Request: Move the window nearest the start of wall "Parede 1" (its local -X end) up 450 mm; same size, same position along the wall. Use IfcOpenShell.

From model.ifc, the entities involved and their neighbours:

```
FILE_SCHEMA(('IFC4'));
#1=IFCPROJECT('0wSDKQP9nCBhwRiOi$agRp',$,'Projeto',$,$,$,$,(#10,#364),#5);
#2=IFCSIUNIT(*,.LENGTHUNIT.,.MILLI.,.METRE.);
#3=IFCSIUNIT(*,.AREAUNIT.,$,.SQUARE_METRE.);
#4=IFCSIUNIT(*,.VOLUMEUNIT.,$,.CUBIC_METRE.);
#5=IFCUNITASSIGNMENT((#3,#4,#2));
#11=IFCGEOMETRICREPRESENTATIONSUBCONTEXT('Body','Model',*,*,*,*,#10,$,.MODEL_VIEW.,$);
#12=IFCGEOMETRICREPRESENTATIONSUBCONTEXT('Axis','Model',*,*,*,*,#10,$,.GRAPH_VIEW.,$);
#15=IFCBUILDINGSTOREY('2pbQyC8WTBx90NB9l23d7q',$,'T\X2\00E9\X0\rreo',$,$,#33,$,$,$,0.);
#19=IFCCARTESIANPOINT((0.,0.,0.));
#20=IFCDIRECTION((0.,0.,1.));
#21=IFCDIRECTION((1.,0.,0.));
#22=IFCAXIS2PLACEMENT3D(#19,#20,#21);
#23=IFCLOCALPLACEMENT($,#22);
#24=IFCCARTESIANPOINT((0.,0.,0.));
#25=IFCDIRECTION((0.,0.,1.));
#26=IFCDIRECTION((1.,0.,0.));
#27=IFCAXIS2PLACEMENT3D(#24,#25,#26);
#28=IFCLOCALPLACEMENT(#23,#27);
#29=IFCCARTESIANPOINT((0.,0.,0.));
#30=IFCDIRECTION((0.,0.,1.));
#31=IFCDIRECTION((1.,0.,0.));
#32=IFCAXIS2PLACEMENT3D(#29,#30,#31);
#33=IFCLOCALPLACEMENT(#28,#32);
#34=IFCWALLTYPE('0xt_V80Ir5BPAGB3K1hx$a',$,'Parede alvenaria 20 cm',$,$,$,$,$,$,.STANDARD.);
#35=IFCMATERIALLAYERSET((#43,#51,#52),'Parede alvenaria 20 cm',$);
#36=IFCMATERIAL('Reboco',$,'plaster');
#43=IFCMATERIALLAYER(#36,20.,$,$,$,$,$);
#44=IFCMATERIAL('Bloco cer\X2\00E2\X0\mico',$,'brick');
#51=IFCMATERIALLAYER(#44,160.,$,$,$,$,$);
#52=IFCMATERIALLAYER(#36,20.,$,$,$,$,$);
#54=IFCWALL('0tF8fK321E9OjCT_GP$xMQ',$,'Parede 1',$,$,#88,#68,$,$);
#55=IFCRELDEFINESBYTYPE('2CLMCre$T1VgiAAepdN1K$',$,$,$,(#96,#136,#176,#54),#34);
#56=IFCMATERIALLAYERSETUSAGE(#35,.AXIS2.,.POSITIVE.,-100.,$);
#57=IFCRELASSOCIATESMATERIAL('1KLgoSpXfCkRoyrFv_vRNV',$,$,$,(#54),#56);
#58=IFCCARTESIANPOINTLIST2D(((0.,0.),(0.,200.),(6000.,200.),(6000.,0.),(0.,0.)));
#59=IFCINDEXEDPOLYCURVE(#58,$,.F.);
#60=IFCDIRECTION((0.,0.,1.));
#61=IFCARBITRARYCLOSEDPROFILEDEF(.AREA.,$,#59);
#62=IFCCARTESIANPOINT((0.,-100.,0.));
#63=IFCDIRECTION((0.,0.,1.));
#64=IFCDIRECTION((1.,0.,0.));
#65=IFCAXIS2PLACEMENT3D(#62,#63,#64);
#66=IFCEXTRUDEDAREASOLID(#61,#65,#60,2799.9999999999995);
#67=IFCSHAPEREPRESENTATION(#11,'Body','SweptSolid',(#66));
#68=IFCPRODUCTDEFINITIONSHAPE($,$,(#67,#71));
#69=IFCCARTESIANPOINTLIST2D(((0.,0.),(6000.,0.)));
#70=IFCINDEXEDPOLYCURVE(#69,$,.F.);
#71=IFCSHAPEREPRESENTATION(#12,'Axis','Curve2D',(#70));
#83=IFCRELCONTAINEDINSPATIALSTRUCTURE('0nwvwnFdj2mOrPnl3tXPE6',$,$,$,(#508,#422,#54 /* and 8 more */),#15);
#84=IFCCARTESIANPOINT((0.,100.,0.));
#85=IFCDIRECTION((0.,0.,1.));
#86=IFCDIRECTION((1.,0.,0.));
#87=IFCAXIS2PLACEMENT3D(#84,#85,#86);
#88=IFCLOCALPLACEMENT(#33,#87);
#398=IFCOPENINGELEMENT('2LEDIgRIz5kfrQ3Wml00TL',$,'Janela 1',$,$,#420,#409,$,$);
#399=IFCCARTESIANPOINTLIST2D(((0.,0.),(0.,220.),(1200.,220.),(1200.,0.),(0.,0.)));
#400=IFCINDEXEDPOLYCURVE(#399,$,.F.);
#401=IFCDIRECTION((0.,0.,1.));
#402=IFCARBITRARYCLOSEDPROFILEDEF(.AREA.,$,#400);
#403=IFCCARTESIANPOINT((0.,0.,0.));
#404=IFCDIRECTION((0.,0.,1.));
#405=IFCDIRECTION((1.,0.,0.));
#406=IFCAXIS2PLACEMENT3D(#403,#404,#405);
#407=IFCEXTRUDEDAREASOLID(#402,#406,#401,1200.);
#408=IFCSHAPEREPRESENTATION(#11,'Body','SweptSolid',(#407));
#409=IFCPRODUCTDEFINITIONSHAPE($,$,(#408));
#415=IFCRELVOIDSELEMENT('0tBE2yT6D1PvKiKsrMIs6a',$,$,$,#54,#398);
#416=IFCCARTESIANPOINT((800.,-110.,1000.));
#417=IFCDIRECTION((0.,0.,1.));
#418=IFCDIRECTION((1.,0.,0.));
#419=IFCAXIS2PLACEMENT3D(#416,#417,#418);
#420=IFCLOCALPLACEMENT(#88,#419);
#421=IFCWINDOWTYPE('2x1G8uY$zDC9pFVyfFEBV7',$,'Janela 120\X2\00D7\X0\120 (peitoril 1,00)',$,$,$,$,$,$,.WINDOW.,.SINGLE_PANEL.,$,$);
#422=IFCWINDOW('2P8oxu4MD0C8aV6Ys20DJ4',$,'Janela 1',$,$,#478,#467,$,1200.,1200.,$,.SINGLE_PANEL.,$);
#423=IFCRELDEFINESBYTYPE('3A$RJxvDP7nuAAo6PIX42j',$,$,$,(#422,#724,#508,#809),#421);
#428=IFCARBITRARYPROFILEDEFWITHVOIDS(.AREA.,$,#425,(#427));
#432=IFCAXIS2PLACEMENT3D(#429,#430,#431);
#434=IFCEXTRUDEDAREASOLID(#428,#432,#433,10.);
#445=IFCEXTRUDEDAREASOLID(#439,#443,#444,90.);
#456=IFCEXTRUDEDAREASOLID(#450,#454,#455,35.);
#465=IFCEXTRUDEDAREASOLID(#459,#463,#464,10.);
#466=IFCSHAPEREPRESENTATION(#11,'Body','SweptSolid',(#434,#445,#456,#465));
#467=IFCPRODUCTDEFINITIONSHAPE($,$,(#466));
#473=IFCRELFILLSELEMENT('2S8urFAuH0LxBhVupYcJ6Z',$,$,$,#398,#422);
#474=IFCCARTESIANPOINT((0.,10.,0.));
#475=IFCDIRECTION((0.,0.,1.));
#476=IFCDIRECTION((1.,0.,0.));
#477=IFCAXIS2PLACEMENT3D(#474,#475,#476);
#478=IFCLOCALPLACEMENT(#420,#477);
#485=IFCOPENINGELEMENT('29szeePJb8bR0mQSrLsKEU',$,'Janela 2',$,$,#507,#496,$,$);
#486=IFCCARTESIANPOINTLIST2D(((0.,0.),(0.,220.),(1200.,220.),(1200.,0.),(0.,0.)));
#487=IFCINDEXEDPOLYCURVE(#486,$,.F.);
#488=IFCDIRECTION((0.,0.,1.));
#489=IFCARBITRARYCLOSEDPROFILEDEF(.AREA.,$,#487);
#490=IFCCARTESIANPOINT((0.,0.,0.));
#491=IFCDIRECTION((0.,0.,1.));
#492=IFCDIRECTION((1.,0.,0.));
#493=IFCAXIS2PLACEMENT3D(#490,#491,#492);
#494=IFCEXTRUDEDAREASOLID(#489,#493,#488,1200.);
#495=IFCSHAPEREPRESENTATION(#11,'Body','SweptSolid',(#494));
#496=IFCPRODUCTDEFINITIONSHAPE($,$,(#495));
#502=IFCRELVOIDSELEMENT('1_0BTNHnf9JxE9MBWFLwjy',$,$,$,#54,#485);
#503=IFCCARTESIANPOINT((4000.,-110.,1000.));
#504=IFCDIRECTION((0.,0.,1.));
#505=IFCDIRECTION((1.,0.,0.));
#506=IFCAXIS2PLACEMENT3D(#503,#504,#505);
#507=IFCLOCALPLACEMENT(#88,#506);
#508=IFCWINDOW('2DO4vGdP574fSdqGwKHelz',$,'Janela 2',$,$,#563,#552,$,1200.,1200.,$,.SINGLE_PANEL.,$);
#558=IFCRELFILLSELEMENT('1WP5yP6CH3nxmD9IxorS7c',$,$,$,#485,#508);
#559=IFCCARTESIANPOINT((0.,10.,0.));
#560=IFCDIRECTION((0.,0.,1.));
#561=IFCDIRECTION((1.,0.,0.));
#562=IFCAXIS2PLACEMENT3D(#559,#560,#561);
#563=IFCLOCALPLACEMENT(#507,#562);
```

```python
import numpy as np
import ifcopenshell
import ifcopenshell.api.geometry
import ifcopenshell.util.placement
import ifcopenshell.util.unit

model = ifcopenshell.open("model.ifc")
unit_scale = ifcopenshell.util.unit.calculate_unit_scale(model)

window = model.by_id(422)
opening = window.FillsVoids[0].RelatingOpeningElement
dz = 0.45 / unit_scale

shift = np.array([0.0, 0.0, dz])
# The window is placed relative to its opening, so it follows when the opening moves.
matrix = ifcopenshell.util.placement.get_local_placement(opening.ObjectPlacement)
matrix[:3, 3] += shift
ifcopenshell.api.geometry.edit_object_placement(
    model, product=opening, matrix=matrix, is_si=False, should_transform_children=True
)

print(f"moved by {dz * unit_scale:+.3f} m")

model.write("model-out.ifc")
```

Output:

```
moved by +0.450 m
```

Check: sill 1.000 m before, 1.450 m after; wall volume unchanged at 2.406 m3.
